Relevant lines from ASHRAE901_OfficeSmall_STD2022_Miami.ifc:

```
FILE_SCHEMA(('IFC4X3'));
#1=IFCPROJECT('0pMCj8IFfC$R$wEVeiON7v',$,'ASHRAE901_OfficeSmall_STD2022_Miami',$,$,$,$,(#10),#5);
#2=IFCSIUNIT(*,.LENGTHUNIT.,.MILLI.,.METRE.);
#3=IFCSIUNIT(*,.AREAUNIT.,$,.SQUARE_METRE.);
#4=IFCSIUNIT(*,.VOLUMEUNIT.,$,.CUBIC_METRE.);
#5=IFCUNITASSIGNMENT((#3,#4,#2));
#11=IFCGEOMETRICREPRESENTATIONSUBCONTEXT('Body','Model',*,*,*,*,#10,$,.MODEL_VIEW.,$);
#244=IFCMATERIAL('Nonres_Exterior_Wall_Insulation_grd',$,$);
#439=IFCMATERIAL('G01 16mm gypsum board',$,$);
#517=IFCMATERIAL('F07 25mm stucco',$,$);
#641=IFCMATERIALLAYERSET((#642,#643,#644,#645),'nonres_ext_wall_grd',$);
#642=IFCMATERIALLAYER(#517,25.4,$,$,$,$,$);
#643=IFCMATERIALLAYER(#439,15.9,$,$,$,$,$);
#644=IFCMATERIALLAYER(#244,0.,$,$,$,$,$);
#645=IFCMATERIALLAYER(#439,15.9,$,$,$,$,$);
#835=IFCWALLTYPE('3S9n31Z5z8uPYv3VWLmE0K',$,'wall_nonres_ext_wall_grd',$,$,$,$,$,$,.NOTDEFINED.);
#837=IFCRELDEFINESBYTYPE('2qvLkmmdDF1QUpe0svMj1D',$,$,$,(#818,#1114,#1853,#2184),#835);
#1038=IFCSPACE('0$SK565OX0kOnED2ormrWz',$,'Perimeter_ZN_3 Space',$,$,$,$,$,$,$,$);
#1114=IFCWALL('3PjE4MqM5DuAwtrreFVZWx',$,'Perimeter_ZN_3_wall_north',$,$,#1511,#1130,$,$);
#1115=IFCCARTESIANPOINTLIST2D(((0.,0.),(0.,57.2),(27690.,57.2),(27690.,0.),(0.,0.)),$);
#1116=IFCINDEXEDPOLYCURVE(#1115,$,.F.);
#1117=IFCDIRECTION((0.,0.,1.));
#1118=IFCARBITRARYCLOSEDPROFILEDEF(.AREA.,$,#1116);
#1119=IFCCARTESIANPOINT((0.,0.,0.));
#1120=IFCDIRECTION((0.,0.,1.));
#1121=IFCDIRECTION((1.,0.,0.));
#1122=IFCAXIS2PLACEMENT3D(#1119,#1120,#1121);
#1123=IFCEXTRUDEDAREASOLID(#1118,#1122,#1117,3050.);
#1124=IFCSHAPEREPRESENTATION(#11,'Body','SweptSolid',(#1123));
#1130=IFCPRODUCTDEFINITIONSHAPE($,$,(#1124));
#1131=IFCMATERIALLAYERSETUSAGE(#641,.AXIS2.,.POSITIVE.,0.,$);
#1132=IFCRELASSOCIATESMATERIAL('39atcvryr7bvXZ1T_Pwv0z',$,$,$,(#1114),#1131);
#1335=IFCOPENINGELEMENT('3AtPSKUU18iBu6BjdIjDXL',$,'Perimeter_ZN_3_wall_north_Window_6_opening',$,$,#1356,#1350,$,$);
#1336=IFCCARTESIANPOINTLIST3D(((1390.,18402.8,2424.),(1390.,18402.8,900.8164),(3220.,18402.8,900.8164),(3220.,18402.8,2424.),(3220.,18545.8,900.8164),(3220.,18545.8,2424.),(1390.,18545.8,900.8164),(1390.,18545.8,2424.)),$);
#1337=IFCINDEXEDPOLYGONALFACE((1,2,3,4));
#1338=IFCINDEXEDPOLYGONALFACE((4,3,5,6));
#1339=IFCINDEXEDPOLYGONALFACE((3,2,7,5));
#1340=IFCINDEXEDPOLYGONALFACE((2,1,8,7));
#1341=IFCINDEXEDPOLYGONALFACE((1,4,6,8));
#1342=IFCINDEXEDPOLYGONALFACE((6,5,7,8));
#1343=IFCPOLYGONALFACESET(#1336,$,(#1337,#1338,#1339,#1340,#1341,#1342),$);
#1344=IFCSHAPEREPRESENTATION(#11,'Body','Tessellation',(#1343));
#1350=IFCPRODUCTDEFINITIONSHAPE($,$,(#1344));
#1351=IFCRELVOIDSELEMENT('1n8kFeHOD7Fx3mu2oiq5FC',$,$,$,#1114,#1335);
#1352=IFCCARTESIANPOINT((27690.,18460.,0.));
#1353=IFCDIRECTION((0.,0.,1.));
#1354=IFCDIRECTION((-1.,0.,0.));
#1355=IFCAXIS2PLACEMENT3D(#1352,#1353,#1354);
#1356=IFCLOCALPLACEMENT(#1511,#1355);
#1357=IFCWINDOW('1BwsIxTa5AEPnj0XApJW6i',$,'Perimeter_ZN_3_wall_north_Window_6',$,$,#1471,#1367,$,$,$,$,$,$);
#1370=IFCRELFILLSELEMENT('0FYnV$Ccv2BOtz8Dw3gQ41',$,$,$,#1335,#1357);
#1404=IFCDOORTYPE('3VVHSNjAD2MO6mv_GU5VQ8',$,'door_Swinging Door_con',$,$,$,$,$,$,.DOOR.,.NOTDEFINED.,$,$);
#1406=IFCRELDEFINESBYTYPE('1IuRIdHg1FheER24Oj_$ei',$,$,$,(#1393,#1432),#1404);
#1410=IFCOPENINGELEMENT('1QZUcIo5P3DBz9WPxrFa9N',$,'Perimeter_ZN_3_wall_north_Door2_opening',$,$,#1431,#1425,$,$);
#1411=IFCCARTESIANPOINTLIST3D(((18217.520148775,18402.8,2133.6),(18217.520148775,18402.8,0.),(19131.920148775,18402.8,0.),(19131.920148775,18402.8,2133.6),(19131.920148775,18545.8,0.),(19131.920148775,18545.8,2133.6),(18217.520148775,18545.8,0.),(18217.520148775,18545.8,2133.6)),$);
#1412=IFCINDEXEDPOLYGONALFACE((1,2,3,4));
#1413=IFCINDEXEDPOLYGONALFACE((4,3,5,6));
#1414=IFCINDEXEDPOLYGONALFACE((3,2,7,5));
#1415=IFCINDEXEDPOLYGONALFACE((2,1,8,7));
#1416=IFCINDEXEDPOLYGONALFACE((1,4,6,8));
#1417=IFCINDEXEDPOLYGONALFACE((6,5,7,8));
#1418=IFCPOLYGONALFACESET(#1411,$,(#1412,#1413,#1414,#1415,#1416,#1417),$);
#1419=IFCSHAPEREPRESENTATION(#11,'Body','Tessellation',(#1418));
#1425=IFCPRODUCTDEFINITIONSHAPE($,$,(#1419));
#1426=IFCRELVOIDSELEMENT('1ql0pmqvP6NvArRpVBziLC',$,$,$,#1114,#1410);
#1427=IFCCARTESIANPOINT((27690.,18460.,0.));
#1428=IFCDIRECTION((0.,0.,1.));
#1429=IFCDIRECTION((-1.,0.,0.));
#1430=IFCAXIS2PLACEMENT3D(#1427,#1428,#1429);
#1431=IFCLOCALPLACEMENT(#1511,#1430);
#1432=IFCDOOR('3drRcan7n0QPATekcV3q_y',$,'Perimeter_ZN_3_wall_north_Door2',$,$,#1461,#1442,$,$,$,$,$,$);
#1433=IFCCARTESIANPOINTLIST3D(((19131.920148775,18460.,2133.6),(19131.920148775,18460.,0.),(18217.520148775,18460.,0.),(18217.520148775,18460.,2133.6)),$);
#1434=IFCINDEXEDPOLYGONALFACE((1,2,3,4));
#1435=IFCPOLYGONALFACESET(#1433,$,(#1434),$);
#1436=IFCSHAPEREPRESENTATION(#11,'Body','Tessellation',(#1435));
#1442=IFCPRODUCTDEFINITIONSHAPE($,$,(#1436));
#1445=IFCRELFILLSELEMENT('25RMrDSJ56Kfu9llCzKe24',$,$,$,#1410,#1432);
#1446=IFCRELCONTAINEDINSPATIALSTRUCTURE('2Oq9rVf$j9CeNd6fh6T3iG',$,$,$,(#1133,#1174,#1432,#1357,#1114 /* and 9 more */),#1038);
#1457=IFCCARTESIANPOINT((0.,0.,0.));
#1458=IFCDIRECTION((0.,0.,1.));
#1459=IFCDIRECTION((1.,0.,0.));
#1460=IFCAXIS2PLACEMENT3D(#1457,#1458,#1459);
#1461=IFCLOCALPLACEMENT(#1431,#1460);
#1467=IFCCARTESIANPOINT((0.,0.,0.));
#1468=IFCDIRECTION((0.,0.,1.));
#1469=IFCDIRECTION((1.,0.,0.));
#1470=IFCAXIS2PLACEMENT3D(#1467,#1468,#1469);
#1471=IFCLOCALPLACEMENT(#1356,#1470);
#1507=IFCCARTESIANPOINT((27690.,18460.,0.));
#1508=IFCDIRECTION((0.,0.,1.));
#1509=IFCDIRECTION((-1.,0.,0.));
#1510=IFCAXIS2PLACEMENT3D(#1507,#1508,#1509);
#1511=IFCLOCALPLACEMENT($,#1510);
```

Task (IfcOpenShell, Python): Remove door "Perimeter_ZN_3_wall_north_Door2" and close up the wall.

```python
import ifcopenshell
import ifcopenshell.api.feature
import ifcopenshell.api.root
import ifcopenshell.geom
import ifcopenshell.util.shape

model = ifcopenshell.open("ASHRAE901_OfficeSmall_STD2022_Miami.ifc")
settings = ifcopenshell.geom.settings()


def volume(element):
    """Net volume in cubic metres, openings subtracted."""
    shape = ifcopenshell.geom.create_shape(settings, element)
    return ifcopenshell.util.shape.get_volume(shape.geometry)


door = model.by_guid("3drRcan7n0QPATekcV3q_y")
opening = door.FillsVoids[0].RelatingOpeningElement
wall = opening.VoidsElements[0].RelatingBuildingElement
before = volume(wall)

ifcopenshell.api.root.remove_product(model, product=door)
ifcopenshell.api.feature.remove_feature(model, feature=opening)

after = volume(wall)

print(f"wall volume {before:.3f} -> {after:.3f} m3")

model.write("ASHRAE901_OfficeSmall_STD2022_Miami_v2.ifc")
```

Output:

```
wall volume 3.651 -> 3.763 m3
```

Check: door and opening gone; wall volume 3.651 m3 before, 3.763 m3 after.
